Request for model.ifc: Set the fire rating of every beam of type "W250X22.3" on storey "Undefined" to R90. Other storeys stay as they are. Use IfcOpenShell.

First a look at what the model holds.

```python
import ifcopenshell
import ifcopenshell.util.element

model = ifcopenshell.open("model.ifc")
print(model.schema)
storey = next(s for s in model.by_type("IfcBuildingStorey") if s.Name == "Undefined")
beams = [e for e in ifcopenshell.util.element.get_decomposition(storey) if e.is_a("IfcBeam")]
seen = {}
for e in beams:
    element_type = ifcopenshell.util.element.get_type(e)
    key = (element_type.Name if element_type != e and element_type else None, ifcopenshell.util.element.get_pset(e, "Pset_BeamCommon", "FireRating"))
    seen[key] = seen.get(key, 0) + 1
for (name, value), count in sorted(seen.items(), key=str):
    print(count, "x", name, "|", value)
```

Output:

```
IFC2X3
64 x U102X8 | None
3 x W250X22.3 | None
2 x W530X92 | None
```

```python
import ifcopenshell
import ifcopenshell.api.pset
import ifcopenshell.util.element

model = ifcopenshell.open("model.ifc")

storey = next(s for s in model.by_type("IfcBuildingStorey") if s.Name == "Undefined")
beams = [e for e in ifcopenshell.util.element.get_decomposition(storey) if e.is_a("IfcBeam")]

count = 0
for e in beams:
    element_type = ifcopenshell.util.element.get_type(e)
    if element_type in (None, e) or element_type.Name != "W250X22.3":
        continue
    found = ifcopenshell.util.element.get_pset(e, "Pset_BeamCommon", should_inherit=False)
    if found:
        pset = model.by_id(found["id"])
        if len(ifcopenshell.util.element.get_elements_by_pset(pset)) > 1:
            pset = ifcopenshell.api.pset.unshare_pset(model, products=[e], pset=pset)[0]
    else:
        pset = ifcopenshell.api.pset.add_pset(model, product=e, name="Pset_BeamCommon")
    ifcopenshell.api.pset.edit_pset(model, pset=pset, properties={"FireRating": "R90"})
    count += 1

print(count, "beams updated")

model.write("model-out.ifc")
```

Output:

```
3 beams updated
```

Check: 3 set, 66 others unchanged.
